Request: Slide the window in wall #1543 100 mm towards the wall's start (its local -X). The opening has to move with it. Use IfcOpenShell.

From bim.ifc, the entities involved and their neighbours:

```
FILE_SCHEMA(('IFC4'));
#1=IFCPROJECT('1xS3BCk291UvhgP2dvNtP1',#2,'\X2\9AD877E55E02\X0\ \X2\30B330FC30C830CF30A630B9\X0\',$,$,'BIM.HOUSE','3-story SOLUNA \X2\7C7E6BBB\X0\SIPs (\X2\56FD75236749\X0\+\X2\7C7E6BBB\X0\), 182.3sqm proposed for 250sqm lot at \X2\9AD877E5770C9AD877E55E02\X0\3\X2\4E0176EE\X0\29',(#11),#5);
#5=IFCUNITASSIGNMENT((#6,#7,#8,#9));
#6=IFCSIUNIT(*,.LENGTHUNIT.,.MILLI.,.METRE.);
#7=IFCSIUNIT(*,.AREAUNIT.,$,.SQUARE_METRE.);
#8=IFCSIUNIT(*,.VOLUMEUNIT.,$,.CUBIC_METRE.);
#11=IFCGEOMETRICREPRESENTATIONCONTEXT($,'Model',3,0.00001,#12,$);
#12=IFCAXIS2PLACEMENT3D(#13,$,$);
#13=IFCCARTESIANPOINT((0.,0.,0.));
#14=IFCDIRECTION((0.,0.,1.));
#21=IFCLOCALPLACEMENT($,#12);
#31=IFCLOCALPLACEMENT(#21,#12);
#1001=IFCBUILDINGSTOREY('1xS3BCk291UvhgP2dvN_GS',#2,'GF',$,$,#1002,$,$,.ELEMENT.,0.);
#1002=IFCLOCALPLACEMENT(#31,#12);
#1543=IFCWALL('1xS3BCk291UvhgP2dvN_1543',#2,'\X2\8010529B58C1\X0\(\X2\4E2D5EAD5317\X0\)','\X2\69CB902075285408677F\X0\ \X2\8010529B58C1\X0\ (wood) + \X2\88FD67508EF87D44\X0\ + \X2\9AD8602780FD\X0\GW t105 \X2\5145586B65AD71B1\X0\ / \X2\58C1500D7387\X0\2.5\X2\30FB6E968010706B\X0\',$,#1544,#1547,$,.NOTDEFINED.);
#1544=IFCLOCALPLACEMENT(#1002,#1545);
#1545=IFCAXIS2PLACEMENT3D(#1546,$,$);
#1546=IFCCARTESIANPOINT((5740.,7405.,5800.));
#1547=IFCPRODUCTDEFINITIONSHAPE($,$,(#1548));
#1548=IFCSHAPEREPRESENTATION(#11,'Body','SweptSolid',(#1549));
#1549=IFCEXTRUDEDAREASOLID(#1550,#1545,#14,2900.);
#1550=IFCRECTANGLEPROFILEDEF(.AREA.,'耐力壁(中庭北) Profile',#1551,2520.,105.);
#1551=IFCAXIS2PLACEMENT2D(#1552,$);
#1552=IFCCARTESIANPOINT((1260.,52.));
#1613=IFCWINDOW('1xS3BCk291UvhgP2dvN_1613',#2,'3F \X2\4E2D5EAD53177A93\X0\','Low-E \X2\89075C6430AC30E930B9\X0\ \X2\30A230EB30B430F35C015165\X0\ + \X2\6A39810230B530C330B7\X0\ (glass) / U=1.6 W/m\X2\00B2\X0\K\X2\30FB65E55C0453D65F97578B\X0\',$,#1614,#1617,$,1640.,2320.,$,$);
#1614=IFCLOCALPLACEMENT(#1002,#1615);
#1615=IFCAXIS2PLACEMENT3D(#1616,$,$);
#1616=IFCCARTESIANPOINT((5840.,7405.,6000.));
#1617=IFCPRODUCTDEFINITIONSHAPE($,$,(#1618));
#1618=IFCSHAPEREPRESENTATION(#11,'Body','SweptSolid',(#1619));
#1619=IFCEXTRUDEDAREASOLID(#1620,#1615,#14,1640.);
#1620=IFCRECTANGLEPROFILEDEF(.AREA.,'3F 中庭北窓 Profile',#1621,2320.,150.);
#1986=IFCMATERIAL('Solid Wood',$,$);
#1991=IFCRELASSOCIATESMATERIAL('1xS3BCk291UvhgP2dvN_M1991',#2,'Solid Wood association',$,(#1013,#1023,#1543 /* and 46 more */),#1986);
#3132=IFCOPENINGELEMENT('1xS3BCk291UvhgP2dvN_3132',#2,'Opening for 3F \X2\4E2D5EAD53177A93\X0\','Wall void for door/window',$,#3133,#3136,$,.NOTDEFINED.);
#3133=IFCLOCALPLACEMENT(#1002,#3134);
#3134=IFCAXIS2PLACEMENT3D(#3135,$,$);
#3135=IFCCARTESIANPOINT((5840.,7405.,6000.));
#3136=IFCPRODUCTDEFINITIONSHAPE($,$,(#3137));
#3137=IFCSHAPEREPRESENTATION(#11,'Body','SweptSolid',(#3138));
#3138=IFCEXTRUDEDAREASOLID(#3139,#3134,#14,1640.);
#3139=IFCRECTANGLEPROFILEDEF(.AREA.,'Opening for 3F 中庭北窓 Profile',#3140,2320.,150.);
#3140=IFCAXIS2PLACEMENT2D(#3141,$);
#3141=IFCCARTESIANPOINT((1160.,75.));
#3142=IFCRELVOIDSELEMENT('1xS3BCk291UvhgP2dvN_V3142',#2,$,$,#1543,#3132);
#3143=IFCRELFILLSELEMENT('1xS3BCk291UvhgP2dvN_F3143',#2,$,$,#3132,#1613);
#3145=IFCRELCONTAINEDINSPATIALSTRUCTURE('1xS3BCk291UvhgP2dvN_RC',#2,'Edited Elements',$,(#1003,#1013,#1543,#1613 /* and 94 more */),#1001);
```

```python
import ifcopenshell
import ifcopenshell.api.geometry
import ifcopenshell.util.placement
import ifcopenshell.util.unit

model = ifcopenshell.open("bim.ifc")
unit_scale = ifcopenshell.util.unit.calculate_unit_scale(model)

window = model.by_id(1613)
opening = window.FillsVoids[0].RelatingOpeningElement
wall = opening.VoidsElements[0].RelatingBuildingElement

wall_matrix = ifcopenshell.util.placement.get_local_placement(wall.ObjectPlacement)
shift = wall_matrix[:3, 0] * -0.1 / unit_scale
before = ifcopenshell.util.placement.get_local_placement(window.ObjectPlacement)[:3, 3].copy()

# The window is not placed relative to its opening, so move both.
for product in (opening, window):
    matrix = ifcopenshell.util.placement.get_local_placement(product.ObjectPlacement)
    matrix[:3, 3] += shift
    ifcopenshell.api.geometry.edit_object_placement(model, product=product, matrix=matrix, is_si=False)

after = ifcopenshell.util.placement.get_local_placement(window.ObjectPlacement)[:3, 3]
print("window moved by", (after - before).round(3) + 0.0)

model.write("bim_rev.ifc")
```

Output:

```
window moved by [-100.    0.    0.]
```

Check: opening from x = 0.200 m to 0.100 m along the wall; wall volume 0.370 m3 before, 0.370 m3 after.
